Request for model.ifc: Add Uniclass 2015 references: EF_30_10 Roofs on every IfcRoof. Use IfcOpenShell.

First a look at what the model holds.

```python
import ifcopenshell

model = ifcopenshell.open("model.ifc")
print(model.schema)
print("classifications:", [c.Name for c in model.by_type("IfcClassification")])
for ifc_class in ("IfcDoor", "IfcRoof", "IfcStair", "IfcWall", "IfcWindow"):
    print(ifc_class, len(model.by_type(ifc_class)))
```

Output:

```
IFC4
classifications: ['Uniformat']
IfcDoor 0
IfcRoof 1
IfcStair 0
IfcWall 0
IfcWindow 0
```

```python
import ifcopenshell
import ifcopenshell.api.classification

model = ifcopenshell.open("model.ifc")

system = ifcopenshell.api.classification.add_classification(model, classification="Uniclass 2015")

codes = {
    "IfcRoof": ("EF_30_10", "Roofs"),
}
for ifc_class, (code, name) in codes.items():
    products = model.by_type(ifc_class)
    ifcopenshell.api.classification.add_reference(
        model, products=products, classification=system, identification=code, name=name
    )
    print(code, len(products))

model.write("model_edited.ifc")
```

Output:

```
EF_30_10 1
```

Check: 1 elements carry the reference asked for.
